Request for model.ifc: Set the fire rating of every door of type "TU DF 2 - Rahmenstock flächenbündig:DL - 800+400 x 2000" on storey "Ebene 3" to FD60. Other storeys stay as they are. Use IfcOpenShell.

First a look at what the model holds.

```python
import ifcopenshell
import ifcopenshell.util.element

model = ifcopenshell.open("model.ifc")
print(model.schema)
storey = next(s for s in model.by_type("IfcBuildingStorey") if s.Name == "Ebene 3")
doors = [e for e in ifcopenshell.util.element.get_decomposition(storey) if e.is_a("IfcDoor")]
seen = {}
for e in doors:
    element_type = ifcopenshell.util.element.get_type(e)
    key = (element_type.Name if element_type != e and element_type else None, ifcopenshell.util.element.get_pset(e, "Pset_DoorCommon", "FireRating"))
    seen[key] = seen.get(key, 0) + 1
for (name, value), count in sorted(seen.items(), key=str):
    print(count, "x", name, "|", value)
```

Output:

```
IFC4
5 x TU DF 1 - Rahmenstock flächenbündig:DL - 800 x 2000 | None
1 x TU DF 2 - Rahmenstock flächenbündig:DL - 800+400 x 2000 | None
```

```python
import ifcopenshell
import ifcopenshell.api.pset
import ifcopenshell.util.element

model = ifcopenshell.open("model.ifc")

storey = next(s for s in model.by_type("IfcBuildingStorey") if s.Name == "Ebene 3")
doors = [e for e in ifcopenshell.util.element.get_decomposition(storey) if e.is_a("IfcDoor")]

count = 0
for e in doors:
    element_type = ifcopenshell.util.element.get_type(e)
    if element_type in (None, e) or element_type.Name != "TU DF 2 - Rahmenstock flächenbündig:DL - 800+400 x 2000":
        continue
    # add_pset returns the element's existing set when there is one.
    pset = ifcopenshell.api.pset.add_pset(model, product=e, name="Pset_DoorCommon")
    ifcopenshell.api.pset.edit_pset(model, pset=pset, properties={"FireRating": "FD60"})
    count += 1

print(count, "doors updated")

model.write("model_edited.ifc")
```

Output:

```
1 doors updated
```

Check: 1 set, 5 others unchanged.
